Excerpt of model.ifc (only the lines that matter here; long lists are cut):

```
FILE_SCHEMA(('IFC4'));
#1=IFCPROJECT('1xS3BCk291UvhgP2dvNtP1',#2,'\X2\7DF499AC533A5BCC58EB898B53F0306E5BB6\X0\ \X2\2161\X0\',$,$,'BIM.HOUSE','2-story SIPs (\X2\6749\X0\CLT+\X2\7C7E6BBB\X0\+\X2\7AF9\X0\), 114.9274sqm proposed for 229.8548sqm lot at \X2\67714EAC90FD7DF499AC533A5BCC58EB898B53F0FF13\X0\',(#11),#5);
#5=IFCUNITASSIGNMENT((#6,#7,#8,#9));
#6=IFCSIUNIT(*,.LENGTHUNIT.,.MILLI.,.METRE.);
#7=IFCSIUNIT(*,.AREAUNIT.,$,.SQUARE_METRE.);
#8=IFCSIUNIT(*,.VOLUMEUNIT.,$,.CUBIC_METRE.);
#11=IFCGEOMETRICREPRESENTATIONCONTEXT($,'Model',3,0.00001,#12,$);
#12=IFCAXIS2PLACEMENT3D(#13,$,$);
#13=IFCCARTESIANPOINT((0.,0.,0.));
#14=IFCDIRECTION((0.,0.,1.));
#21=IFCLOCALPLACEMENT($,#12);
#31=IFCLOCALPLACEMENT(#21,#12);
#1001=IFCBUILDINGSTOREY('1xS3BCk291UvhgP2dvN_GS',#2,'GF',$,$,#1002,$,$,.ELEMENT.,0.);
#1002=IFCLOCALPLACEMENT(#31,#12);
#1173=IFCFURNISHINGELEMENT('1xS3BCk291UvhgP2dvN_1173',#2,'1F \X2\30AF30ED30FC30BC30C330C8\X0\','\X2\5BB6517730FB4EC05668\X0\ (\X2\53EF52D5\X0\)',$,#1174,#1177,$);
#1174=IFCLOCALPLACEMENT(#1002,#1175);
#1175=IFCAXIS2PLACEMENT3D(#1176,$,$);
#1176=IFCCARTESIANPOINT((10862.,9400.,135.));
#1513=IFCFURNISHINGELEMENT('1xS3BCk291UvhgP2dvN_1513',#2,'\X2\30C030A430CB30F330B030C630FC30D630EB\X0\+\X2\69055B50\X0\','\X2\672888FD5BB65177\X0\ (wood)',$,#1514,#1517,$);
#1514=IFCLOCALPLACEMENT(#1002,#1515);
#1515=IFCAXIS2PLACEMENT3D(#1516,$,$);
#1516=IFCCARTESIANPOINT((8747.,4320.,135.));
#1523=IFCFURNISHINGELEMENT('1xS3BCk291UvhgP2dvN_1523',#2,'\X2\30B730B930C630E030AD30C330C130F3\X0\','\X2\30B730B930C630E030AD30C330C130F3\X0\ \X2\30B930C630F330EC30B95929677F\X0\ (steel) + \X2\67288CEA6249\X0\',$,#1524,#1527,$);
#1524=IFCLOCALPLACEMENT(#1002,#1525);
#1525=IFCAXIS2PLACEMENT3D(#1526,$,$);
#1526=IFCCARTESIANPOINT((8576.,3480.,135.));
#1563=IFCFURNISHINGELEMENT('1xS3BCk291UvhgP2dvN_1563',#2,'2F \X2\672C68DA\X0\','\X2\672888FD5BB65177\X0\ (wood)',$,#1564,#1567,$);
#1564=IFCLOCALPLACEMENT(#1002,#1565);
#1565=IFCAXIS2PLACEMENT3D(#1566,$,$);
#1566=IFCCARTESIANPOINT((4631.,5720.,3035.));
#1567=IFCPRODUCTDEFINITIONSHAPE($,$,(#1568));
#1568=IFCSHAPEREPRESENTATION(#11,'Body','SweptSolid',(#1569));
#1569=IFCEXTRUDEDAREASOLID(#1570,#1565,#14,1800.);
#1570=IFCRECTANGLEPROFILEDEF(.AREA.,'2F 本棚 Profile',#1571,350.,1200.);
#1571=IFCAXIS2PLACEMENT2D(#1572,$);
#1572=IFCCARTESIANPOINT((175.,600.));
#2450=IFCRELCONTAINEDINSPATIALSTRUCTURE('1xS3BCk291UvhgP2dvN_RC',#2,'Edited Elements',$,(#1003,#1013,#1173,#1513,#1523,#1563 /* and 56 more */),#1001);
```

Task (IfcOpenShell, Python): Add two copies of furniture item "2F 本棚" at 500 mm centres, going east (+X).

```python
import numpy as np
import ifcopenshell
import ifcopenshell.api.geometry
import ifcopenshell.api.root
import ifcopenshell.util.element
import ifcopenshell.util.placement
import ifcopenshell.util.unit

model = ifcopenshell.open("model.ifc")
unit_scale = ifcopenshell.util.unit.calculate_unit_scale(model)


def reuse_history(source, copy):
    """copy_class also copies each property set's owner history, people and application; keep the originals."""
    for rel in copy.IsDefinedBy:
        if rel.is_a("IfcRelDefinesByProperties") and (history := rel.RelatingPropertyDefinition.OwnerHistory):
            rel.RelatingPropertyDefinition.OwnerHistory = source.OwnerHistory
            ifcopenshell.util.element.remove_deep2(model, history)


source = model.by_id(1563)
base = ifcopenshell.util.placement.get_local_placement(source.ObjectPlacement)
step = np.array([1.0, 0.0, 0.0]) * 0.5 / unit_scale

for i in range(1, 3):
    copy = ifcopenshell.api.root.copy_class(model, product=source)
    copy.Representation = ifcopenshell.util.element.copy_deep(
        model, source.Representation, exclude=["IfcGeometricRepresentationContext", "IfcRepresentationMap"]
    )
    reuse_history(source, copy)
    matrix = base.copy()
    matrix[:3, 3] += i * step
    print("added at", matrix[:3, 3].round(3) + 0.0)
    ifcopenshell.api.geometry.edit_object_placement(model, product=copy, matrix=matrix, is_si=False)

model.write("model_v2.ifc")
```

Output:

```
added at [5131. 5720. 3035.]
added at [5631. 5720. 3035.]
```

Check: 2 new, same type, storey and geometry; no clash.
